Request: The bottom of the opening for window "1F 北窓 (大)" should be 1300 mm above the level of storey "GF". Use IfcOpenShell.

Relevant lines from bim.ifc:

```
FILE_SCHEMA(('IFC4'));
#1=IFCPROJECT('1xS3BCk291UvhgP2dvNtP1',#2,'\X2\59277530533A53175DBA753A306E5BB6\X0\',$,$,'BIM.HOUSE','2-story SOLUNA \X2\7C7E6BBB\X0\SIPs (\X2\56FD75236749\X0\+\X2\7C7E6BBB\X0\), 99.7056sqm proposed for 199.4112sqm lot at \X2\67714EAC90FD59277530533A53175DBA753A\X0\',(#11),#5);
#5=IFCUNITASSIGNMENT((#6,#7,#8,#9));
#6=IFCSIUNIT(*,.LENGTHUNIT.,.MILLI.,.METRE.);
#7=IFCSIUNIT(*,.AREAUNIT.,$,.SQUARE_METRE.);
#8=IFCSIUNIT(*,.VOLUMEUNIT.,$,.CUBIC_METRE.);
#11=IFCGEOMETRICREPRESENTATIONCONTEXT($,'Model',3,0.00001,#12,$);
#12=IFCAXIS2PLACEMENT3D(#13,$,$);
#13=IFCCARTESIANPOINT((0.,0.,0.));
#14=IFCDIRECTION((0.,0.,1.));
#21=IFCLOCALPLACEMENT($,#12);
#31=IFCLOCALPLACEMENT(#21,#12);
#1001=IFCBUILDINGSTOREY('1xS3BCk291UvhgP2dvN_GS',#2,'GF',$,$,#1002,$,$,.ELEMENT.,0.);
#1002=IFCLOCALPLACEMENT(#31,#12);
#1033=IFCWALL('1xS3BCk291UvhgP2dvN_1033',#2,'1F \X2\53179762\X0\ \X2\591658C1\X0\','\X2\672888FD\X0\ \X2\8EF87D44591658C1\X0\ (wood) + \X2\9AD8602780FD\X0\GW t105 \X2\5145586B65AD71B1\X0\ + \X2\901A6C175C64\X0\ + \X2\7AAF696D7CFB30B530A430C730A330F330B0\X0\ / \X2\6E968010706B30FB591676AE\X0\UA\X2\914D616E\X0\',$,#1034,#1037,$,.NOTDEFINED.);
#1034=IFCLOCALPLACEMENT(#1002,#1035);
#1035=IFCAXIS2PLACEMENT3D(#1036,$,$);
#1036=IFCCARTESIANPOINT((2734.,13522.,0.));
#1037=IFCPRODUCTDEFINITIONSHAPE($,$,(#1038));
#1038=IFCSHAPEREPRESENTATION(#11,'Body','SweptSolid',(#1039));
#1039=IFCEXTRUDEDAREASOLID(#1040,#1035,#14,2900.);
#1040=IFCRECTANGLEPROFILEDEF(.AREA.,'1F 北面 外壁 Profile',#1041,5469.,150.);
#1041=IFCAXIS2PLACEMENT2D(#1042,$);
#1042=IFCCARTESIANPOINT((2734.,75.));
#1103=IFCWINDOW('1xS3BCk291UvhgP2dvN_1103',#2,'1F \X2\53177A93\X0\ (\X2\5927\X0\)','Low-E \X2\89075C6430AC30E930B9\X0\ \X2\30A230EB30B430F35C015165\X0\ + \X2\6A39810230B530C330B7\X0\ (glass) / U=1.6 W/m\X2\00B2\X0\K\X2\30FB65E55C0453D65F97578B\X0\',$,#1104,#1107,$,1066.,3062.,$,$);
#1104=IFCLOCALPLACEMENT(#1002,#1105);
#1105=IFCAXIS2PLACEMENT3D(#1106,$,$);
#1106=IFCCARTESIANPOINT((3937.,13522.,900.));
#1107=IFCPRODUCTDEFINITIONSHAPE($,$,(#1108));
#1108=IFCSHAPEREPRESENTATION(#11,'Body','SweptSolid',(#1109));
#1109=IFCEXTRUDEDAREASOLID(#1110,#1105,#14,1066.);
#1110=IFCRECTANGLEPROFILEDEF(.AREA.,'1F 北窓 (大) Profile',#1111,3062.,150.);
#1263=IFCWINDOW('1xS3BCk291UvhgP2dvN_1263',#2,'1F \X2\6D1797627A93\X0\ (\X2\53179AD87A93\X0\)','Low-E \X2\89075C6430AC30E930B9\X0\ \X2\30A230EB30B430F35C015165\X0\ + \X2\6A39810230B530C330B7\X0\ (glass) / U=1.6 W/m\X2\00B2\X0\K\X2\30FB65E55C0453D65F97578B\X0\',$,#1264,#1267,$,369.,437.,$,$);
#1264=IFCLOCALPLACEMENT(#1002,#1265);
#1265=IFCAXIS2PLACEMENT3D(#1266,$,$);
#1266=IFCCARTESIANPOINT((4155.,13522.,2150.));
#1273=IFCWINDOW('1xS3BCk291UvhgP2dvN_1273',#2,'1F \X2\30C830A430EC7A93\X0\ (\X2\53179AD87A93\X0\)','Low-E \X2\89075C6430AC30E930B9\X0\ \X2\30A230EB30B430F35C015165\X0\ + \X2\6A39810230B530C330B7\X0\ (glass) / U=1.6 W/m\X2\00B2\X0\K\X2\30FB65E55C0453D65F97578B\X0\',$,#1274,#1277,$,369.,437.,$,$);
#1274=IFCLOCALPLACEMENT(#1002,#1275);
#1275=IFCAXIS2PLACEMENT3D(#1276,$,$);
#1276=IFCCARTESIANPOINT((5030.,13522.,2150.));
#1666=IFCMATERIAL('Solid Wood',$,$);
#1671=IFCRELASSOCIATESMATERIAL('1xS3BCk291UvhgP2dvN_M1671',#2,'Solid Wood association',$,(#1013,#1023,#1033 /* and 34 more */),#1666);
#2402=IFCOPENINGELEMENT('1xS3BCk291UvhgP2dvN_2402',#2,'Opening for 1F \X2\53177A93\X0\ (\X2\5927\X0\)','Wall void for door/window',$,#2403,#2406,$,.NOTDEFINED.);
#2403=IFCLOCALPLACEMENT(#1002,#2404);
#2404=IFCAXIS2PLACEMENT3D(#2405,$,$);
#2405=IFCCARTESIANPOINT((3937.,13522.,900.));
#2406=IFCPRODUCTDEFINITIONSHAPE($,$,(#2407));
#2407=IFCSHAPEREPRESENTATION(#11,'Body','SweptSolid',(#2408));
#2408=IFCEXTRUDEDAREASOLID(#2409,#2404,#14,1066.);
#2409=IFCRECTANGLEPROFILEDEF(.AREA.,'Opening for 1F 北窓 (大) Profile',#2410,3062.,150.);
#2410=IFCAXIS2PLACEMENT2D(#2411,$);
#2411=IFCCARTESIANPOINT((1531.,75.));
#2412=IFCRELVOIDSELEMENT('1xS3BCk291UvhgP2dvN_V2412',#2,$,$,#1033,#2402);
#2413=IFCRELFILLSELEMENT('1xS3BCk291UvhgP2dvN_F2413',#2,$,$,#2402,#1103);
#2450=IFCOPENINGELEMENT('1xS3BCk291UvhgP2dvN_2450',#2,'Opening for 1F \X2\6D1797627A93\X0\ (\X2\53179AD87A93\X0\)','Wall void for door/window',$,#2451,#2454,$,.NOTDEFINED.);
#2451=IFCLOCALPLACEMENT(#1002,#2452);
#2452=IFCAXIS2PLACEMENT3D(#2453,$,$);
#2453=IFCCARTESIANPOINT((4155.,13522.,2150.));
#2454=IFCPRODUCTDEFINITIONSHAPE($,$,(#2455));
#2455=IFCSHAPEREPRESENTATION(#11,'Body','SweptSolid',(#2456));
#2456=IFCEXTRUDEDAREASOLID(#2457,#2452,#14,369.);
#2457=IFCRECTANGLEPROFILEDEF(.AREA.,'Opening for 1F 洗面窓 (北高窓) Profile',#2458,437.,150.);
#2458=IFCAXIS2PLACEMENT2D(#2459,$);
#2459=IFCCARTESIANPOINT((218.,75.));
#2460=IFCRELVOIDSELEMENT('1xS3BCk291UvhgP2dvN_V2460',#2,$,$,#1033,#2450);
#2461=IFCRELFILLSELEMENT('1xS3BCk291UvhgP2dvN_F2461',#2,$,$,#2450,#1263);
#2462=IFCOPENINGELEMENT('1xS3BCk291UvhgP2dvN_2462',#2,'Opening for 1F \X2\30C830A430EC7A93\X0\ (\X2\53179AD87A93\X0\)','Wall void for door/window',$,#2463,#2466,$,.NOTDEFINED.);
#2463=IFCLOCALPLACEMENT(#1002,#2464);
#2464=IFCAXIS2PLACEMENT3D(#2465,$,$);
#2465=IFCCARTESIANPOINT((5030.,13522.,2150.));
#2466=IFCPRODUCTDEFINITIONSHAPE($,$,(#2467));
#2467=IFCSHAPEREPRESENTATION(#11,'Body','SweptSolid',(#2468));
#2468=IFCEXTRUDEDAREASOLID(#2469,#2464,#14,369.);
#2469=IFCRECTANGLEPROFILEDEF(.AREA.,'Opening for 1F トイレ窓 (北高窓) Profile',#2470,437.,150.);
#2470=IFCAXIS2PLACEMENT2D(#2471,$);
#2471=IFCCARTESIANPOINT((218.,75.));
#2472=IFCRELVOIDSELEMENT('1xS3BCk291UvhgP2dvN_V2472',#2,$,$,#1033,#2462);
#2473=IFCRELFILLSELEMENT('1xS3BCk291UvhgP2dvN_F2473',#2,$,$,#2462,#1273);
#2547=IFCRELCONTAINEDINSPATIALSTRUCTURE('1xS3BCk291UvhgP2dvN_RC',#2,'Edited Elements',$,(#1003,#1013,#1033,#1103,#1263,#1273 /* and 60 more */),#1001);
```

```python
import numpy as np
import ifcopenshell
import ifcopenshell.api.geometry
import ifcopenshell.geom
import ifcopenshell.util.element
import ifcopenshell.util.placement
import ifcopenshell.util.shape
import ifcopenshell.util.unit

model = ifcopenshell.open("bim.ifc")
unit_scale = ifcopenshell.util.unit.calculate_unit_scale(model)

window = model.by_guid("1xS3BCk291UvhgP2dvN_1103")
opening = window.FillsVoids[0].RelatingOpeningElement
storey = ifcopenshell.util.element.get_container(window, ifc_class="IfcBuildingStorey")
level = ifcopenshell.util.placement.get_local_placement(storey.ObjectPlacement)[2, 3]

# The opening's origin need not be at the sill, so measure its lowest point.
shape = ifcopenshell.geom.create_shape(ifcopenshell.geom.settings(), opening)
bottom = ifcopenshell.util.shape.get_shape_bottom_elevation(shape, shape.geometry) / unit_scale
dz = level + 1300.0 - bottom

shift = np.array([0.0, 0.0, dz])
# The window is not placed relative to its opening, so move both.
for product in (opening, window):
    matrix = ifcopenshell.util.placement.get_local_placement(product.ObjectPlacement)
    matrix[:3, 3] += shift
    ifcopenshell.api.geometry.edit_object_placement(model, product=product, matrix=matrix, is_si=False)

print(f"moved by {dz * unit_scale:+.3f} m")

model.write("bim_edited.ifc")
```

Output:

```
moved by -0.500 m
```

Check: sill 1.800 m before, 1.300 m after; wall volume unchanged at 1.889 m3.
